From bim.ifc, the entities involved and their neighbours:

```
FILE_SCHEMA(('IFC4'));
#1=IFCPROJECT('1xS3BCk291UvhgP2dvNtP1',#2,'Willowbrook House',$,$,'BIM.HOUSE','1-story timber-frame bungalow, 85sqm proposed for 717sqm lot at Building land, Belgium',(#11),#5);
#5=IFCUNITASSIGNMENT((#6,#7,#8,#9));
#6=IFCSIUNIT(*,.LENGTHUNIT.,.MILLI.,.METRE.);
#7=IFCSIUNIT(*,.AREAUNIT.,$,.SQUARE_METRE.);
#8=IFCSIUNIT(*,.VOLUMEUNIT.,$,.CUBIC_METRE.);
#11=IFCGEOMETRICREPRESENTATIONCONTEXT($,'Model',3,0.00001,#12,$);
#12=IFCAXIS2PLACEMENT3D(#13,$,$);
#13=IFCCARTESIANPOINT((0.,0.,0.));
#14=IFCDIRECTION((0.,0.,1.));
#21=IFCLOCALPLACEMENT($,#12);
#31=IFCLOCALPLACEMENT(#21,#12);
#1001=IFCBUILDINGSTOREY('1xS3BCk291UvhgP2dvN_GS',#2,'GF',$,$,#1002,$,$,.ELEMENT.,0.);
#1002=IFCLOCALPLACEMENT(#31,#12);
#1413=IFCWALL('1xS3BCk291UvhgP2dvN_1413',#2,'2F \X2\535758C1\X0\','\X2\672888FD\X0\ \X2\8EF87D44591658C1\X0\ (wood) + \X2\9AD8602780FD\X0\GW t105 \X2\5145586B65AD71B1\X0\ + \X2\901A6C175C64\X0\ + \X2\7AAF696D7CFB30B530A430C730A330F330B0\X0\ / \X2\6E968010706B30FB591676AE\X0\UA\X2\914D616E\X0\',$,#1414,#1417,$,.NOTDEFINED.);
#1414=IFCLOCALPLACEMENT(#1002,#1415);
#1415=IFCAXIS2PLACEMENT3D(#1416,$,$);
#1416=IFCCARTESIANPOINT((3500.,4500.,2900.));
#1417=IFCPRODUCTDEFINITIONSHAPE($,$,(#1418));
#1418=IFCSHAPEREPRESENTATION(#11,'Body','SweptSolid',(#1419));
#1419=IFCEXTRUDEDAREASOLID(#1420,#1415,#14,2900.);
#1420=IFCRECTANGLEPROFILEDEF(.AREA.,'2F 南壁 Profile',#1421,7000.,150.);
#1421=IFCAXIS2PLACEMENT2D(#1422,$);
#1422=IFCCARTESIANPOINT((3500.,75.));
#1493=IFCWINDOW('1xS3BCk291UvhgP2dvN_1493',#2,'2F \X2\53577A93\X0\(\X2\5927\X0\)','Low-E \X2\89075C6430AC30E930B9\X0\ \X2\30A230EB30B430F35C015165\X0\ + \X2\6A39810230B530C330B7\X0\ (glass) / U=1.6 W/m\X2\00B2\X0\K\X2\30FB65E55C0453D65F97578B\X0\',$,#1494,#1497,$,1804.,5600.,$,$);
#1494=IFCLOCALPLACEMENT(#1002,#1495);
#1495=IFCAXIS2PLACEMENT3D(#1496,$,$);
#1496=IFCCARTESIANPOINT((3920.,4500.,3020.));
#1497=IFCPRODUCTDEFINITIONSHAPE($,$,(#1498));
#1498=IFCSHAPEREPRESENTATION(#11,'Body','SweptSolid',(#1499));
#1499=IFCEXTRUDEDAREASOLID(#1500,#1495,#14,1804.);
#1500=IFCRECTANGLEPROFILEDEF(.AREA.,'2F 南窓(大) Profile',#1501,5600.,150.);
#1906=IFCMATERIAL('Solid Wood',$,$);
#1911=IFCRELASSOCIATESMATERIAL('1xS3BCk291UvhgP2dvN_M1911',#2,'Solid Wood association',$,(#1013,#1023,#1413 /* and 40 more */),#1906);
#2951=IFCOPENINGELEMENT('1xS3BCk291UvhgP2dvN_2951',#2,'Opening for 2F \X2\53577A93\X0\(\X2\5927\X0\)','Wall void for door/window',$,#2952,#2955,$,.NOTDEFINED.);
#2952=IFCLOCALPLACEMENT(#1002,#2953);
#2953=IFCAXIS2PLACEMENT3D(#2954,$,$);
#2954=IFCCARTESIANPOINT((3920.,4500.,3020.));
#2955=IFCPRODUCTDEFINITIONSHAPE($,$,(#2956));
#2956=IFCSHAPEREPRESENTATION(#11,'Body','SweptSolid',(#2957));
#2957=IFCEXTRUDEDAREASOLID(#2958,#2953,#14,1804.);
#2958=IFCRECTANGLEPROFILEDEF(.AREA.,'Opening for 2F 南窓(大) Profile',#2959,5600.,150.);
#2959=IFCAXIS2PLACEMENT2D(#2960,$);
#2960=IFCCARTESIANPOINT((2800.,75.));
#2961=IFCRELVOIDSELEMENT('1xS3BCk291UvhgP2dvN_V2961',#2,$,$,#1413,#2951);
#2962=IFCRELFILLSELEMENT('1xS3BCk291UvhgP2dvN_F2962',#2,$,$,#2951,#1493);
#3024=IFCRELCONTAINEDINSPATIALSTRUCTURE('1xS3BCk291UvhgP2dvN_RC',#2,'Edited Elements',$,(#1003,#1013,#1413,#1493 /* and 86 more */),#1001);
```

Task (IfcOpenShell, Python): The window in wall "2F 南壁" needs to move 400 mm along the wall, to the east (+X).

```python
import ifcopenshell
import ifcopenshell.api.geometry
import ifcopenshell.util.placement

model = ifcopenshell.open("bim.ifc")

window = model.by_id(1493)
opening = window.FillsVoids[0].RelatingOpeningElement
wall = opening.VoidsElements[0].RelatingBuildingElement

wall_matrix = ifcopenshell.util.placement.get_local_placement(wall.ObjectPlacement)
shift = wall_matrix[:3, 0] * 400.0
before = ifcopenshell.util.placement.get_local_placement(window.ObjectPlacement)[:3, 3].copy()

# The window is not placed relative to its opening, so move both.
for product in (opening, window):
    matrix = ifcopenshell.util.placement.get_local_placement(product.ObjectPlacement)
    matrix[:3, 3] += shift
    ifcopenshell.api.geometry.edit_object_placement(model, product=product, matrix=matrix, is_si=False)

after = ifcopenshell.util.placement.get_local_placement(window.ObjectPlacement)[:3, 3]
print("window moved by", (after - before).round(3) + 0.0)

model.write("bim_edited.ifc")
```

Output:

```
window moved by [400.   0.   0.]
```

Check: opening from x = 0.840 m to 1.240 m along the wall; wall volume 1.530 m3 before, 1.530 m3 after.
